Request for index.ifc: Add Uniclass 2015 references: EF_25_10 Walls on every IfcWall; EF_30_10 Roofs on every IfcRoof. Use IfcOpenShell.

First a look at what the model holds.

```python
import ifcopenshell

model = ifcopenshell.open("index.ifc")
print(model.schema)
print("classifications:", [c.Name for c in model.by_type("IfcClassification")])
for ifc_class in ("IfcDoor", "IfcRoof", "IfcStair", "IfcWall", "IfcWindow"):
    print(ifc_class, len(model.by_type(ifc_class)))
```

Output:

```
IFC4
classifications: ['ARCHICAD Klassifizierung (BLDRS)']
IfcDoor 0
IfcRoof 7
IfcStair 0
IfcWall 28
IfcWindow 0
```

```python
import ifcopenshell
import ifcopenshell.api.classification

model = ifcopenshell.open("index.ifc")

system = ifcopenshell.api.classification.add_classification(model, classification="Uniclass 2015")

codes = {
    "IfcWall": ("EF_25_10", "Walls"),
    "IfcRoof": ("EF_30_10", "Roofs"),
}
for ifc_class, (code, name) in codes.items():
    products = model.by_type(ifc_class)
    ifcopenshell.api.classification.add_reference(
        model, products=products, classification=system, identification=code, name=name
    )
    print(code, len(products))

model.write("index_updated.ifc")
```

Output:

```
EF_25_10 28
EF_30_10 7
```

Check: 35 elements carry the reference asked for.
